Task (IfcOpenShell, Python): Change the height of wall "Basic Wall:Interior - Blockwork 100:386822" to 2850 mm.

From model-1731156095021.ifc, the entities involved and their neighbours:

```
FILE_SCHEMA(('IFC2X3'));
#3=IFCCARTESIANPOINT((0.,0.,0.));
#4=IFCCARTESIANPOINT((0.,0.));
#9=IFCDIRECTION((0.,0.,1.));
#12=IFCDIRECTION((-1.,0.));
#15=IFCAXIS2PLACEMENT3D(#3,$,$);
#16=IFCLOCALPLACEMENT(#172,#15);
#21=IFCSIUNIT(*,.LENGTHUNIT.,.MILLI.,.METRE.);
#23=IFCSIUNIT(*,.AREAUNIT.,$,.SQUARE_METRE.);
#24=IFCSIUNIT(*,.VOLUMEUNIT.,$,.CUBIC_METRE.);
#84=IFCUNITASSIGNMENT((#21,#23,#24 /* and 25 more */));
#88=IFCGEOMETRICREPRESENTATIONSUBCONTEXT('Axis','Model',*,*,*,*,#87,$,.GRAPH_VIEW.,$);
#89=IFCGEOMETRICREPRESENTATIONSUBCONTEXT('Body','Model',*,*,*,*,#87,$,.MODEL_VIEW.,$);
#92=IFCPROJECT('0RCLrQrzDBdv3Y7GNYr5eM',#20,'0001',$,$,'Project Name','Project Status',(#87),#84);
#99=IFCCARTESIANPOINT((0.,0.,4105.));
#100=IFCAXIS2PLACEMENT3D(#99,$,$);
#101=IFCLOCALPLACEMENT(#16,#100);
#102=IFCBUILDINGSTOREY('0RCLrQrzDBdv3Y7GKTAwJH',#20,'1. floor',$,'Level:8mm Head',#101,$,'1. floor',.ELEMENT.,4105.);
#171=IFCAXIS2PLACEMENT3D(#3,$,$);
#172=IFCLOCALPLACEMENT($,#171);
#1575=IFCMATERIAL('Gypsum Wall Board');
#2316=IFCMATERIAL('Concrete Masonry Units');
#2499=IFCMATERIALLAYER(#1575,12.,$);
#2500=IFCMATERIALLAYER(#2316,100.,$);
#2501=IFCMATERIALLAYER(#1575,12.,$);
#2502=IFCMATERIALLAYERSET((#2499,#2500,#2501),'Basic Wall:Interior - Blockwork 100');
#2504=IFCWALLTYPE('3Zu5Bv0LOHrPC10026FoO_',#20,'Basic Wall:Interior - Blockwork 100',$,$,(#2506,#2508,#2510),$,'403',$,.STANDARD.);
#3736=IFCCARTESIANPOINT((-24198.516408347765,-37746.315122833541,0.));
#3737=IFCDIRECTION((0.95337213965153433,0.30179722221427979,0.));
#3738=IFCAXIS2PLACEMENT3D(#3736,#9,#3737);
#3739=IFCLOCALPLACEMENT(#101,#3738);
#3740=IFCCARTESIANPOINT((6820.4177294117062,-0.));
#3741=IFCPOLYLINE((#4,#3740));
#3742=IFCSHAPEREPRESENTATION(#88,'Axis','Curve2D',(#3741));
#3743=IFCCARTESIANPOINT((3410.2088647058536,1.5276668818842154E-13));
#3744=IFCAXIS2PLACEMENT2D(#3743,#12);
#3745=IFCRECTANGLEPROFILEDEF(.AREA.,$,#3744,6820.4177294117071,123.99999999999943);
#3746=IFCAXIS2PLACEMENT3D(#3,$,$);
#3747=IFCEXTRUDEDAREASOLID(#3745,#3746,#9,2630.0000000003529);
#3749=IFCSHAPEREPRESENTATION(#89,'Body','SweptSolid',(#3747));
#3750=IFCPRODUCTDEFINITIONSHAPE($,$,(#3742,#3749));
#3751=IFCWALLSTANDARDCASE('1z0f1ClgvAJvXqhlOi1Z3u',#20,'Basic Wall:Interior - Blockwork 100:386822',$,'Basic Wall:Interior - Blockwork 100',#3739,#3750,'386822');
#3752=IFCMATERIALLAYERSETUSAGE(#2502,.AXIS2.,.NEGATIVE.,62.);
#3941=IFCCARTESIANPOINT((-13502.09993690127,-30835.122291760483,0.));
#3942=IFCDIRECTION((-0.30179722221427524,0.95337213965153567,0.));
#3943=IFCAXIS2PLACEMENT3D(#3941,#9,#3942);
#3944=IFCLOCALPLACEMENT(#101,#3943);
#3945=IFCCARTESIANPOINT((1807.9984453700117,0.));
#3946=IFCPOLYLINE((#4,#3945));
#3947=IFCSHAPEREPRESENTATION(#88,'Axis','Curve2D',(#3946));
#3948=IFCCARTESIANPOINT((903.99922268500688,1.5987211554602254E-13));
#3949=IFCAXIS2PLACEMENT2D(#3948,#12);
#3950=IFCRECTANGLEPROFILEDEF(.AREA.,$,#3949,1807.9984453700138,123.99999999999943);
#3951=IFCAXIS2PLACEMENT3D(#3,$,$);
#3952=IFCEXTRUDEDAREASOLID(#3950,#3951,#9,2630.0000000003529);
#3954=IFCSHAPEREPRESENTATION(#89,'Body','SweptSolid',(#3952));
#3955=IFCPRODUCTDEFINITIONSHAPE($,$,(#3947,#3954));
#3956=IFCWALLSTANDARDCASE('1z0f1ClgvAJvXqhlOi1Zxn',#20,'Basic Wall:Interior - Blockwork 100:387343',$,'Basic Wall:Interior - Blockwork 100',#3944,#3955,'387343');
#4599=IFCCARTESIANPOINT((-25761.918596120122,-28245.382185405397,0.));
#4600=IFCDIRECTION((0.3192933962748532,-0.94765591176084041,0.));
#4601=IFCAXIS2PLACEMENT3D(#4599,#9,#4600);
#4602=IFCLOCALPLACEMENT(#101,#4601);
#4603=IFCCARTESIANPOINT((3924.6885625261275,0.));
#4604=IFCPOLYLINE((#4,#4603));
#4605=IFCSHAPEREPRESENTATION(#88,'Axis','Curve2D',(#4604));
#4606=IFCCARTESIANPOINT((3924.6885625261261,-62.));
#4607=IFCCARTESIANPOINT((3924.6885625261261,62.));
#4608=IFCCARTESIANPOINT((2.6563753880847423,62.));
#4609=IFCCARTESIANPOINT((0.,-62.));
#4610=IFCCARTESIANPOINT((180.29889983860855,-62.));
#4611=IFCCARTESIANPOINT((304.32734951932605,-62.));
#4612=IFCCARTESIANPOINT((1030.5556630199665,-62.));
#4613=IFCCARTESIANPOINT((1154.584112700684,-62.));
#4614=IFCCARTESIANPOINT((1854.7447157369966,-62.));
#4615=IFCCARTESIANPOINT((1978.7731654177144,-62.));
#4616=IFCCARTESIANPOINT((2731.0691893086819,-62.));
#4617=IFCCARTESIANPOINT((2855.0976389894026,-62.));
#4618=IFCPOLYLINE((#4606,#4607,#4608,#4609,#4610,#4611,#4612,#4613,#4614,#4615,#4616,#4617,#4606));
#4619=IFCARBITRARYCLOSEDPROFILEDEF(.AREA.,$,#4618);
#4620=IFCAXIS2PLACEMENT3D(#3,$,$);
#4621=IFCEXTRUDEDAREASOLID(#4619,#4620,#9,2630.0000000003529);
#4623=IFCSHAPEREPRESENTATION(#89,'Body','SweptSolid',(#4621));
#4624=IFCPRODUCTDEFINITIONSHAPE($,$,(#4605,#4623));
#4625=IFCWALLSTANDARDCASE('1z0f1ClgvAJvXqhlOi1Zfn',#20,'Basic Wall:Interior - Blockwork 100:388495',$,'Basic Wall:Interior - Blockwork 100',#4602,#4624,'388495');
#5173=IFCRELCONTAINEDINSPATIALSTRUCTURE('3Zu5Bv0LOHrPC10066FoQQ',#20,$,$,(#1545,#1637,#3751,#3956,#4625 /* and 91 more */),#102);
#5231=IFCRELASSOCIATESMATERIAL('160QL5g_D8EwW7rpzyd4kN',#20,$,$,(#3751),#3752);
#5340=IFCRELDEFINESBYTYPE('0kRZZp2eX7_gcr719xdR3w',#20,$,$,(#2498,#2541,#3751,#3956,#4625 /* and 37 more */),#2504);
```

```python
import ifcopenshell
import ifcopenshell.geom
import ifcopenshell.util.representation
import ifcopenshell.util.shape
import ifcopenshell.util.unit

model = ifcopenshell.open("model-1731156095021.ifc")
unit_scale = ifcopenshell.util.unit.calculate_unit_scale(model)
settings = ifcopenshell.geom.settings()


def volume(element):
    """Net volume in cubic metres, openings subtracted."""
    shape = ifcopenshell.geom.create_shape(settings, element)
    return ifcopenshell.util.shape.get_volume(shape.geometry)


wall = model.by_id(3751)
before = volume(wall)

body = ifcopenshell.util.representation.get_representation(wall, "Model", "Body")
solid = body.Items[0]
old_height = solid.Depth
solid.Depth = 2.85 / unit_scale
after = volume(wall)

print(f"height {old_height:g} -> {solid.Depth:g}, volume {before:.3f} -> {after:.3f} m3")

model.write("model-1731156095021_rev.ifc")
```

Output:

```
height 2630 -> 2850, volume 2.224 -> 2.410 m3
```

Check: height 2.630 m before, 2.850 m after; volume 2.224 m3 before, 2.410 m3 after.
